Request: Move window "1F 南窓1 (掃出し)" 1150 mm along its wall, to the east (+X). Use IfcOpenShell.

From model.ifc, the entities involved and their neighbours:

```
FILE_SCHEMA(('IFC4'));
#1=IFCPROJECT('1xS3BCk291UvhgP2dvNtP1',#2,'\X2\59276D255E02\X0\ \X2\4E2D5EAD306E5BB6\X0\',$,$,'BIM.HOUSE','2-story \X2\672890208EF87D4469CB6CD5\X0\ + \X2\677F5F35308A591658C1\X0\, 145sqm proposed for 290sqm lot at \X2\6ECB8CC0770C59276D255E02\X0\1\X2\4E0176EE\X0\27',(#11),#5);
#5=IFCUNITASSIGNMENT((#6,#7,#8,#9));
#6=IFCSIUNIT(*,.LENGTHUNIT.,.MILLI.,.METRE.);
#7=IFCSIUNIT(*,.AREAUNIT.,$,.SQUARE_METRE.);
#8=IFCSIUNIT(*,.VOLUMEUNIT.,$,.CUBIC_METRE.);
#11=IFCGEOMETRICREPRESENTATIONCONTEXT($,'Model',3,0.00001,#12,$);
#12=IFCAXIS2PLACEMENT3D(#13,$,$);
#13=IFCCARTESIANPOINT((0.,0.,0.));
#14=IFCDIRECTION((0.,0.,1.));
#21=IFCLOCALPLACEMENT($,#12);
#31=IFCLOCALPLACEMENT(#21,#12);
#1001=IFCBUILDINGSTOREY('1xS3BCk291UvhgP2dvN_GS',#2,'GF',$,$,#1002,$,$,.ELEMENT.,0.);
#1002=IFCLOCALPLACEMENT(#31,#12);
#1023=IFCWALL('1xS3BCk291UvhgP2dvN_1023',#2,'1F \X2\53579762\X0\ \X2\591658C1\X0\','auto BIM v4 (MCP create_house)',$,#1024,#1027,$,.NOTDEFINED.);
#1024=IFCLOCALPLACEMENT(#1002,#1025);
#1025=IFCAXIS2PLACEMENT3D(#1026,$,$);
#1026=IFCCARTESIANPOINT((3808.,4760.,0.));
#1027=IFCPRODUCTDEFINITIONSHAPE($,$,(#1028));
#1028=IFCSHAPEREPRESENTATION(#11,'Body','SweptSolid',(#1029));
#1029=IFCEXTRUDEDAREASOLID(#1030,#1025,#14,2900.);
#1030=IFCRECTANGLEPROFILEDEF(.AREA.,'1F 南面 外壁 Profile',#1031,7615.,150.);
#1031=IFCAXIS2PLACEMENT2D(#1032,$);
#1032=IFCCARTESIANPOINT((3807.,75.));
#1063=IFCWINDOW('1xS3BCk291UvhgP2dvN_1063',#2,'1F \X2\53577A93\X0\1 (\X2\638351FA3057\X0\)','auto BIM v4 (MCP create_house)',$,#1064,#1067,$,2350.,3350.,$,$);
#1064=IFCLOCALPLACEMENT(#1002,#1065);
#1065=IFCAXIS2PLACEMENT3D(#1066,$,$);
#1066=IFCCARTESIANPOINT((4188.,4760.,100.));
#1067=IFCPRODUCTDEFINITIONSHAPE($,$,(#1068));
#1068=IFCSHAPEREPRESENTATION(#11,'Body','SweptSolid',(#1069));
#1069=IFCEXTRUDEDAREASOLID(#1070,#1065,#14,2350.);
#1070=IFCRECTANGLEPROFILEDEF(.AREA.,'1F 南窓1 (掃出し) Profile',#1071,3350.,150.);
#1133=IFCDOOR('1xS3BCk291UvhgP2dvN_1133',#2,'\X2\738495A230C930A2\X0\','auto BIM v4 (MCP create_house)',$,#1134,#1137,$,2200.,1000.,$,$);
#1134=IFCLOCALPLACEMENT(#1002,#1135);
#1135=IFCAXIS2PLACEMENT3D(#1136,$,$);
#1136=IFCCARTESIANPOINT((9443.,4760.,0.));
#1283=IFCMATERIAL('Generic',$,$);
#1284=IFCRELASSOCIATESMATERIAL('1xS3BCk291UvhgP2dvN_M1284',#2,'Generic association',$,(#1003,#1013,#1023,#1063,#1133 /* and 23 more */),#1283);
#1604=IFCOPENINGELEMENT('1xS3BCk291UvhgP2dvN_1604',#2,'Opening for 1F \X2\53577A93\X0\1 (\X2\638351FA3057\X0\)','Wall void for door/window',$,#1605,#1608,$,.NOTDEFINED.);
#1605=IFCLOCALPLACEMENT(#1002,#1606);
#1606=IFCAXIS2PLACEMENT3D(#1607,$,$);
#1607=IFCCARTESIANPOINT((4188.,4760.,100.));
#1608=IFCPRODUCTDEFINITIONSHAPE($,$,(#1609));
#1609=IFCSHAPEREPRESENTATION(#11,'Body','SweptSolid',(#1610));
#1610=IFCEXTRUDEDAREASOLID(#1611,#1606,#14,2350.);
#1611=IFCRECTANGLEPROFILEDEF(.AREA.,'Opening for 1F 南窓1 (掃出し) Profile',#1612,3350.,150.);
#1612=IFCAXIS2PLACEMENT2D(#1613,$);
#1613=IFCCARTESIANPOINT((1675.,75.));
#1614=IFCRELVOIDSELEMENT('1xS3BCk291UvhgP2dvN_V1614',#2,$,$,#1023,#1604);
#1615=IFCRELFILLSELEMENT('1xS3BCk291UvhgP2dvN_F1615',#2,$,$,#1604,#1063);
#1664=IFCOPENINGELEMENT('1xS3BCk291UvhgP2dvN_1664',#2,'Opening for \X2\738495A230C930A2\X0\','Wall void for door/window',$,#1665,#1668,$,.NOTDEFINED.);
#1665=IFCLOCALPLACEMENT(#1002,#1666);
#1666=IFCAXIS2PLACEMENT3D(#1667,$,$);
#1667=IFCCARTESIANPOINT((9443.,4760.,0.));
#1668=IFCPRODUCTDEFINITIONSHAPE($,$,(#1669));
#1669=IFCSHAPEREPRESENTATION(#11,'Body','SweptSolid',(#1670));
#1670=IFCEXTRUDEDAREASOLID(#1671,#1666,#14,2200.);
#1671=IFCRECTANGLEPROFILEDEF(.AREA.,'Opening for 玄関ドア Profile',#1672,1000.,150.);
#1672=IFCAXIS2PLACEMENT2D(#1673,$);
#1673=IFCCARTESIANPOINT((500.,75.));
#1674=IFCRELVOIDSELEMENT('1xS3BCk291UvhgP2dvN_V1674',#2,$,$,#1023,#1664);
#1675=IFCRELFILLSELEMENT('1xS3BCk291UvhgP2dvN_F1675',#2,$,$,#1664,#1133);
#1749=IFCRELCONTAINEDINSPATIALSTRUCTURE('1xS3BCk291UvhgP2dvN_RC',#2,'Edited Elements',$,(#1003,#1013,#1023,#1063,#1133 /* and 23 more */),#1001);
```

```python
import ifcopenshell
import ifcopenshell.api.geometry
import ifcopenshell.util.placement
import ifcopenshell.util.unit

model = ifcopenshell.open("model.ifc")
unit_scale = ifcopenshell.util.unit.calculate_unit_scale(model)

window = model.by_guid("1xS3BCk291UvhgP2dvN_1063")
opening = window.FillsVoids[0].RelatingOpeningElement
wall = opening.VoidsElements[0].RelatingBuildingElement

wall_matrix = ifcopenshell.util.placement.get_local_placement(wall.ObjectPlacement)
shift = wall_matrix[:3, 0] * 1.15 / unit_scale
before = ifcopenshell.util.placement.get_local_placement(window.ObjectPlacement)[:3, 3].copy()

# The window is not placed relative to its opening, so move both.
for product in (opening, window):
    matrix = ifcopenshell.util.placement.get_local_placement(product.ObjectPlacement)
    matrix[:3, 3] += shift
    ifcopenshell.api.geometry.edit_object_placement(model, product=product, matrix=matrix, is_si=False)

after = ifcopenshell.util.placement.get_local_placement(window.ObjectPlacement)[:3, 3]
print("window moved by", (after - before).round(3) + 0.0)

model.write("model_rev.ifc")
```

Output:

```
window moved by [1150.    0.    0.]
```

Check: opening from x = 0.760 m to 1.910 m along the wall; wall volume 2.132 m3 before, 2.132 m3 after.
